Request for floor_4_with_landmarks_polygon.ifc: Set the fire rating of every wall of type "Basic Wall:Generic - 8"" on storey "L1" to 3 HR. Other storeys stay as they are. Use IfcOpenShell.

First a look at what the model holds.

```python
import ifcopenshell
import ifcopenshell.util.element

model = ifcopenshell.open("floor_4_with_landmarks_polygon.ifc")
print(model.schema)
storey = next(s for s in model.by_type("IfcBuildingStorey") if s.Name == "L1")
walls = [e for e in ifcopenshell.util.element.get_decomposition(storey) if e.is_a("IfcWall")]
seen = {}
for e in walls:
    element_type = ifcopenshell.util.element.get_type(e)
    key = (element_type.Name if element_type != e and element_type else None, ifcopenshell.util.element.get_pset(e, "Pset_WallCommon", "FireRating"))
    seen[key] = seen.get(key, 0) + 1
for (name, value), count in sorted(seen.items(), key=str):
    print(count, "x", name, "|", value)
```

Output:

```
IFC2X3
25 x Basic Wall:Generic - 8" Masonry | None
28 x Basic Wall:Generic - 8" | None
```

```python
import ifcopenshell
import ifcopenshell.api.pset
import ifcopenshell.util.element

model = ifcopenshell.open("floor_4_with_landmarks_polygon.ifc")

storey = next(s for s in model.by_type("IfcBuildingStorey") if s.Name == "L1")
walls = [e for e in ifcopenshell.util.element.get_decomposition(storey) if e.is_a("IfcWall")]

count = 0
for e in walls:
    element_type = ifcopenshell.util.element.get_type(e)
    if element_type in (None, e) or element_type.Name != 'Basic Wall:Generic - 8"':
        continue
    # add_pset returns the element's existing set when there is one.
    pset = ifcopenshell.api.pset.add_pset(model, product=e, name="Pset_WallCommon")
    ifcopenshell.api.pset.edit_pset(model, pset=pset, properties={"FireRating": "3 HR"})
    count += 1

print(count, "walls updated")

model.write("floor_4_with_landmarks_polygon-out.ifc")
```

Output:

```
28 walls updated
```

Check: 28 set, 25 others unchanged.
